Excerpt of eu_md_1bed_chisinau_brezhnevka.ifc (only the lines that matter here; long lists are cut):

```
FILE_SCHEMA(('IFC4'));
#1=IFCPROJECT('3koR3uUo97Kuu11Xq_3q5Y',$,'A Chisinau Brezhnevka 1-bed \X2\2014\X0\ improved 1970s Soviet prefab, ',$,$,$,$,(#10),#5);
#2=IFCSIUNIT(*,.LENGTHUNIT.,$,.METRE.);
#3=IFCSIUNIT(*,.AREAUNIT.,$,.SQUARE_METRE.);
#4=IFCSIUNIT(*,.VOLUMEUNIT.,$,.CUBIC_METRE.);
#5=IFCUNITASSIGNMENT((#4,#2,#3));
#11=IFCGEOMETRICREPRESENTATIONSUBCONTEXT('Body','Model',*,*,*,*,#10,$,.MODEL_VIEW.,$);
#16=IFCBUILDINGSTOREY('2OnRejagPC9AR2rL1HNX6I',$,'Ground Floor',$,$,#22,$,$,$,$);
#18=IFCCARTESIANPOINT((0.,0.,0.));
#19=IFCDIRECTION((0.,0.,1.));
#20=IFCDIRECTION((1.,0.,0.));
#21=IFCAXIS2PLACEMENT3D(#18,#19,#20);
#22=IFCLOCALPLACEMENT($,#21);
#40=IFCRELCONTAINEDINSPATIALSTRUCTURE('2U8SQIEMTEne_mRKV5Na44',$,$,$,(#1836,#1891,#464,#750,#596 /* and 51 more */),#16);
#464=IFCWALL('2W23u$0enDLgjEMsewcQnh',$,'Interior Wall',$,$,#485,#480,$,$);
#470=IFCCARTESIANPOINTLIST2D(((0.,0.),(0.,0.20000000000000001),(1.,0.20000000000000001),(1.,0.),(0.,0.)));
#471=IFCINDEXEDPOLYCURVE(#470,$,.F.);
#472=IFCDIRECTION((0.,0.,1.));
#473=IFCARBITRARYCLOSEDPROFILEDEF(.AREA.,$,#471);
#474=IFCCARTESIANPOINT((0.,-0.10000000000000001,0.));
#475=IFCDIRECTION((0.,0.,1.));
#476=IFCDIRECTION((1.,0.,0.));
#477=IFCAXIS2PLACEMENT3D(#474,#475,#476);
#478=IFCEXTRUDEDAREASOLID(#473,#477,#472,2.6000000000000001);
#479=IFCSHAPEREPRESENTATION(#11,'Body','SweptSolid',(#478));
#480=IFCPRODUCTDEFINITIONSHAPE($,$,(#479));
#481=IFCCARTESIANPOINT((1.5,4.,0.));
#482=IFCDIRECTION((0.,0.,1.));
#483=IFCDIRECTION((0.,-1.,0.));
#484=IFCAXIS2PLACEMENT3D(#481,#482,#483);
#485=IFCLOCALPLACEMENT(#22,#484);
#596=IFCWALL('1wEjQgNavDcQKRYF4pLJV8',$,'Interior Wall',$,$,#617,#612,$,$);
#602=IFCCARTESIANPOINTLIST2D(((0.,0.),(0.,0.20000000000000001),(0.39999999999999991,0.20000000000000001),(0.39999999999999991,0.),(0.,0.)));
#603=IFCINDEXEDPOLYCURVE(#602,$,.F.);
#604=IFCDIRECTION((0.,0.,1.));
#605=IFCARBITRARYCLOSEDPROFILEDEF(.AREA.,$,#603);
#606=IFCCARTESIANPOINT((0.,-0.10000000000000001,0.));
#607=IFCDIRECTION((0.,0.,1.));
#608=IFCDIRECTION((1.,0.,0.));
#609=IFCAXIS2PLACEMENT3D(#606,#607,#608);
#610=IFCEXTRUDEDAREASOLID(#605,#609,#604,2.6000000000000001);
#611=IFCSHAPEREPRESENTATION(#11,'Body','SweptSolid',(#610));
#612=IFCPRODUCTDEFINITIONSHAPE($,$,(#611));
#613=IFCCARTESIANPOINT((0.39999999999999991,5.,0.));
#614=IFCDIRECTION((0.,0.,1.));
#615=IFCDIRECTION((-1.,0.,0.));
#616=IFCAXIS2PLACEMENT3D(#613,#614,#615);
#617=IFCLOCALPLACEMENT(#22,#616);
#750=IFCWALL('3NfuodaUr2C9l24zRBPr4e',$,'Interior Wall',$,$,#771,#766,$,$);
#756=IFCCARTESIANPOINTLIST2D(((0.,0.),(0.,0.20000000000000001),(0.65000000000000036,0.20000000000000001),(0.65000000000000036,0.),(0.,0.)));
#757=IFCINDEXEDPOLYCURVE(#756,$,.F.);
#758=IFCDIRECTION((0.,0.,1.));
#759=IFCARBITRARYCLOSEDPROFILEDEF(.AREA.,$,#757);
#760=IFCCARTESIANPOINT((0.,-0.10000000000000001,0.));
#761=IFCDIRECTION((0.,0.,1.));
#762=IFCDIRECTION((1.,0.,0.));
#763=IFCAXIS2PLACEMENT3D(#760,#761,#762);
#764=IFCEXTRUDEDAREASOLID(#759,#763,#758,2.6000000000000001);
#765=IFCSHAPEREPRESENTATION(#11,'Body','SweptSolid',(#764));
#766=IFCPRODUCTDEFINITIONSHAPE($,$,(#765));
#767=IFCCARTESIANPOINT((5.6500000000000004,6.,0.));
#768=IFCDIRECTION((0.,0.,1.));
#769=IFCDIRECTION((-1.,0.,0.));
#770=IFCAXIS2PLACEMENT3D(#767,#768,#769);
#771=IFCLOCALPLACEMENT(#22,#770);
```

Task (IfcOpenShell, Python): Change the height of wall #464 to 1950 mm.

```python
import ifcopenshell
import ifcopenshell.geom
import ifcopenshell.util.representation
import ifcopenshell.util.shape
import ifcopenshell.util.unit

model = ifcopenshell.open("eu_md_1bed_chisinau_brezhnevka.ifc")
unit_scale = ifcopenshell.util.unit.calculate_unit_scale(model)
settings = ifcopenshell.geom.settings()


def volume(element):
    """Net volume in cubic metres, openings subtracted."""
    shape = ifcopenshell.geom.create_shape(settings, element)
    return ifcopenshell.util.shape.get_volume(shape.geometry)


wall = model.by_id(464)
before = volume(wall)

body = ifcopenshell.util.representation.get_representation(wall, "Model", "Body")
solid = body.Items[0]
old_height = solid.Depth
solid.Depth = 1.95 / unit_scale
after = volume(wall)

print(f"height {old_height:g} -> {solid.Depth:g}, volume {before:.3f} -> {after:.3f} m3")

model.write("eu_md_1bed_chisinau_brezhnevka-out.ifc")
```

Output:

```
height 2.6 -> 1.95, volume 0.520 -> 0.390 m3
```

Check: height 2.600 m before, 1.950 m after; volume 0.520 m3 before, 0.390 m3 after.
